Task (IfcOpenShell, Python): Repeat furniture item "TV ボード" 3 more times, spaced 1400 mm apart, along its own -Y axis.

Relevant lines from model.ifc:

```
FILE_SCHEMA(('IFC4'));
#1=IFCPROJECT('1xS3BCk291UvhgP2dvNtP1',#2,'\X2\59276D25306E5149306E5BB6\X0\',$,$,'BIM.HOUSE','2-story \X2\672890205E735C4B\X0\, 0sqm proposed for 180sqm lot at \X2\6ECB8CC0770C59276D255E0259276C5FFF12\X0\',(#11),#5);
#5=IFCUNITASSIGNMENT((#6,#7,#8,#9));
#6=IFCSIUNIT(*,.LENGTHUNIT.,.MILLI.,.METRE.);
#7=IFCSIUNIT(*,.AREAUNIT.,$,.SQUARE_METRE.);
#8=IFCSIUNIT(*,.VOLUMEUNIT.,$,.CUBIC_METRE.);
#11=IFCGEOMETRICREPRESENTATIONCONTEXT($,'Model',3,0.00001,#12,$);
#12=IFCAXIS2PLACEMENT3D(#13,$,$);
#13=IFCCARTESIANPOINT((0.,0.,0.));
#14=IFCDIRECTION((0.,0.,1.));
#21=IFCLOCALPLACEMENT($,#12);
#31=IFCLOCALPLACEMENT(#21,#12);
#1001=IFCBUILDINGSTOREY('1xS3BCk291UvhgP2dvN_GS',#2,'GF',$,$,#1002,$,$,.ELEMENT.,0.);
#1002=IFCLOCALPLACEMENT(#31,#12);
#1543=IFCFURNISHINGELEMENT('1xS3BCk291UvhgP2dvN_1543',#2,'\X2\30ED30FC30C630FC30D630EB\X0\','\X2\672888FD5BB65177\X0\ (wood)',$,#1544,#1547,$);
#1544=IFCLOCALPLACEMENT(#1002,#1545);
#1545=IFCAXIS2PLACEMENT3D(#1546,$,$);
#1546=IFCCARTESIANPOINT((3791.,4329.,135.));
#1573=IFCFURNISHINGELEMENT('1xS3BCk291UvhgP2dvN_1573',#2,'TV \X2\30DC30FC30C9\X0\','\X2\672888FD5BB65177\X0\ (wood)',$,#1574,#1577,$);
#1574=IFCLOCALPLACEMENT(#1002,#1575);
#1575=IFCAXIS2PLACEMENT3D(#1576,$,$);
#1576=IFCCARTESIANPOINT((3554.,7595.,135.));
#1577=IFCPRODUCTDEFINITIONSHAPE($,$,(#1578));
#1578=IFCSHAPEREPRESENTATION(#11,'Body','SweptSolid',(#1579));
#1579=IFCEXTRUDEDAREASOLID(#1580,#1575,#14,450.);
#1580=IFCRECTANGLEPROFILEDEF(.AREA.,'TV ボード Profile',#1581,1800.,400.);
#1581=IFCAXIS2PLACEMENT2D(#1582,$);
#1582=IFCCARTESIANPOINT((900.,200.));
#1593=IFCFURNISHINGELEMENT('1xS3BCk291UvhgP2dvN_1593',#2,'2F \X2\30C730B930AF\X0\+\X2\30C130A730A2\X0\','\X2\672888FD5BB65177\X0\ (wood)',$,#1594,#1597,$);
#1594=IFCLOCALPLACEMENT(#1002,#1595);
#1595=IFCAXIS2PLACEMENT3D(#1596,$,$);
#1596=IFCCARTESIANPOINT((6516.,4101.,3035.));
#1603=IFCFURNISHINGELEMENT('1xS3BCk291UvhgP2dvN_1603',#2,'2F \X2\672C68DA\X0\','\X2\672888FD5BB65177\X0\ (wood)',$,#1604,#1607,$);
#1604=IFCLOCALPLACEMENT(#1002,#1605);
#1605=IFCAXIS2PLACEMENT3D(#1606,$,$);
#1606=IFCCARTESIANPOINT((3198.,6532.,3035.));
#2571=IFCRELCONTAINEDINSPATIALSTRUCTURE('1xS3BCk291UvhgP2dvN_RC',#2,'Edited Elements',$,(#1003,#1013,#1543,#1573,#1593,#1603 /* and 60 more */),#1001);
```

```python
import ifcopenshell
import ifcopenshell.api.geometry
import ifcopenshell.api.root
import ifcopenshell.util.element
import ifcopenshell.util.placement
import ifcopenshell.util.unit

model = ifcopenshell.open("model.ifc")
unit_scale = ifcopenshell.util.unit.calculate_unit_scale(model)


def reuse_history(source, copy):
    """copy_class also copies each property set's owner history, people and application; keep the originals."""
    for rel in copy.IsDefinedBy:
        if rel.is_a("IfcRelDefinesByProperties") and (history := rel.RelatingPropertyDefinition.OwnerHistory):
            rel.RelatingPropertyDefinition.OwnerHistory = source.OwnerHistory
            ifcopenshell.util.element.remove_deep2(model, history)


source = model.by_guid("1xS3BCk291UvhgP2dvN_1573")
base = ifcopenshell.util.placement.get_local_placement(source.ObjectPlacement)
step = -base[:3, 1] * 1.4 / unit_scale

for i in range(1, 4):
    copy = ifcopenshell.api.root.copy_class(model, product=source)
    copy.Representation = ifcopenshell.util.element.copy_deep(
        model, source.Representation, exclude=["IfcGeometricRepresentationContext", "IfcRepresentationMap"]
    )
    reuse_history(source, copy)
    matrix = base.copy()
    matrix[:3, 3] += i * step
    print("added at", matrix[:3, 3].round(3) + 0.0)
    ifcopenshell.api.geometry.edit_object_placement(model, product=copy, matrix=matrix, is_si=False)

model.write("model_edited.ifc")
```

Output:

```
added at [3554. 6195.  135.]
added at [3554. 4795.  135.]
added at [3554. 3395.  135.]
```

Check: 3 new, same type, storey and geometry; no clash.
